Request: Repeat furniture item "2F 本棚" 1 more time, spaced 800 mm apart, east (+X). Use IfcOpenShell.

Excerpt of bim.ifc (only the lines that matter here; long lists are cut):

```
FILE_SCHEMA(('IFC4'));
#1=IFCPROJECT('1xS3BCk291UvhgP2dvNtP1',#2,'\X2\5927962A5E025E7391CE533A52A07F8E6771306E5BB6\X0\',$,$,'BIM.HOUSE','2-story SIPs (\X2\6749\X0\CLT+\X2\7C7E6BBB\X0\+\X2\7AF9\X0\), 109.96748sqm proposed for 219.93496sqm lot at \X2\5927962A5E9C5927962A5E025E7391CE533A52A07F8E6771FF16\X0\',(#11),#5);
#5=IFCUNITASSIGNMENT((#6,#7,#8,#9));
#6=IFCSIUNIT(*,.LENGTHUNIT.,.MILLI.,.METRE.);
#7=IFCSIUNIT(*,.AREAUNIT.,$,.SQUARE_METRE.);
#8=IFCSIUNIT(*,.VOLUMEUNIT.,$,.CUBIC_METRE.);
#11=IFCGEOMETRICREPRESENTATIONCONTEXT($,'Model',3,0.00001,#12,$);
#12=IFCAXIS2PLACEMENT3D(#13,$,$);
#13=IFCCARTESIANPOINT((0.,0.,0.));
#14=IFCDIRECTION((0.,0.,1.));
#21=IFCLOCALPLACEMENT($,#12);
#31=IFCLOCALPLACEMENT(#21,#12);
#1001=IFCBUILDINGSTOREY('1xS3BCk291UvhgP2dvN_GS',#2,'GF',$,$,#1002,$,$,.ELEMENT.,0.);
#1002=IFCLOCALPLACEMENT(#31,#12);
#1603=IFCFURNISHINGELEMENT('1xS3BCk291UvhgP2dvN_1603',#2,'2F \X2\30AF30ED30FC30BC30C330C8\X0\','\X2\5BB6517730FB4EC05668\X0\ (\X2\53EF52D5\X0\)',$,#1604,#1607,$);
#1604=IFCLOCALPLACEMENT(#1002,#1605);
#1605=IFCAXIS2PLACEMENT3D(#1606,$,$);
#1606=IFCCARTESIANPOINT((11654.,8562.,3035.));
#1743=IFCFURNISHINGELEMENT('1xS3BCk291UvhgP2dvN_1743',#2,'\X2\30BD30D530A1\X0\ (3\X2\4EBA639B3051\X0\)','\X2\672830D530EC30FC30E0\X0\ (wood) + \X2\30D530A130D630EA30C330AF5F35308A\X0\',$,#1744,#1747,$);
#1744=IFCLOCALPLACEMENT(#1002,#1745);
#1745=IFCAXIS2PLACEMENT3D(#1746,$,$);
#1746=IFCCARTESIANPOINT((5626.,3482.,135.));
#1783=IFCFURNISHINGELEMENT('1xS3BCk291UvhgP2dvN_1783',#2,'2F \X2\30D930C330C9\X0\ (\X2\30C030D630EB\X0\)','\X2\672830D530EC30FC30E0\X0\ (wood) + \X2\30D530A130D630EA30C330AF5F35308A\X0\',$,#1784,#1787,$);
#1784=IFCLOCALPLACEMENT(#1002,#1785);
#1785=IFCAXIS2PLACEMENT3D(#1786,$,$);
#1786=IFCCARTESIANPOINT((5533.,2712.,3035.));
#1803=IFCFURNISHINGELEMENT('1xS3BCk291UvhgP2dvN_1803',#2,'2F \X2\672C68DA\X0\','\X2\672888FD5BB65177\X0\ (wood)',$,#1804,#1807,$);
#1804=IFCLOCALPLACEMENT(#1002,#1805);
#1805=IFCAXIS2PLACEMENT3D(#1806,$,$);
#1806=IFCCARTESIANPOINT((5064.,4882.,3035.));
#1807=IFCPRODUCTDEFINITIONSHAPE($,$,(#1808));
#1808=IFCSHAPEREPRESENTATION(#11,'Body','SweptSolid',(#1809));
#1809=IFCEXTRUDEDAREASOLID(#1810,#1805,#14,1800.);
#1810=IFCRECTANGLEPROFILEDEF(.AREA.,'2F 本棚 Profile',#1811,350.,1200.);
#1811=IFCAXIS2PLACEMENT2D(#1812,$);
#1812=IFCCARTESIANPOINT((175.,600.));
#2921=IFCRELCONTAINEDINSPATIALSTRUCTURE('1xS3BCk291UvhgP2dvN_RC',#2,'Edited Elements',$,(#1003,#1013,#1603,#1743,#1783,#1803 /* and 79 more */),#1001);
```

```python
import numpy as np
import ifcopenshell
import ifcopenshell.api.geometry
import ifcopenshell.api.root
import ifcopenshell.util.element
import ifcopenshell.util.placement
import ifcopenshell.util.unit

model = ifcopenshell.open("bim.ifc")
unit_scale = ifcopenshell.util.unit.calculate_unit_scale(model)


def reuse_history(source, copy):
    """copy_class also copies each property set's owner history, people and application; keep the originals."""
    for rel in copy.IsDefinedBy:
        if rel.is_a("IfcRelDefinesByProperties") and (history := rel.RelatingPropertyDefinition.OwnerHistory):
            rel.RelatingPropertyDefinition.OwnerHistory = source.OwnerHistory
            ifcopenshell.util.element.remove_deep2(model, history)


source = model.by_guid("1xS3BCk291UvhgP2dvN_1803")
base = ifcopenshell.util.placement.get_local_placement(source.ObjectPlacement)
step = np.array([1.0, 0.0, 0.0]) * 0.8 / unit_scale

for i in range(1, 2):
    copy = ifcopenshell.api.root.copy_class(model, product=source)
    copy.Representation = ifcopenshell.util.element.copy_deep(
        model, source.Representation, exclude=["IfcGeometricRepresentationContext", "IfcRepresentationMap"]
    )
    reuse_history(source, copy)
    matrix = base.copy()
    matrix[:3, 3] += i * step
    print("added at", matrix[:3, 3].round(3) + 0.0)
    ifcopenshell.api.geometry.edit_object_placement(model, product=copy, matrix=matrix, is_si=False)

model.write("bim_v2.ifc")
```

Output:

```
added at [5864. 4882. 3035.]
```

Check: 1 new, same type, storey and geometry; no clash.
